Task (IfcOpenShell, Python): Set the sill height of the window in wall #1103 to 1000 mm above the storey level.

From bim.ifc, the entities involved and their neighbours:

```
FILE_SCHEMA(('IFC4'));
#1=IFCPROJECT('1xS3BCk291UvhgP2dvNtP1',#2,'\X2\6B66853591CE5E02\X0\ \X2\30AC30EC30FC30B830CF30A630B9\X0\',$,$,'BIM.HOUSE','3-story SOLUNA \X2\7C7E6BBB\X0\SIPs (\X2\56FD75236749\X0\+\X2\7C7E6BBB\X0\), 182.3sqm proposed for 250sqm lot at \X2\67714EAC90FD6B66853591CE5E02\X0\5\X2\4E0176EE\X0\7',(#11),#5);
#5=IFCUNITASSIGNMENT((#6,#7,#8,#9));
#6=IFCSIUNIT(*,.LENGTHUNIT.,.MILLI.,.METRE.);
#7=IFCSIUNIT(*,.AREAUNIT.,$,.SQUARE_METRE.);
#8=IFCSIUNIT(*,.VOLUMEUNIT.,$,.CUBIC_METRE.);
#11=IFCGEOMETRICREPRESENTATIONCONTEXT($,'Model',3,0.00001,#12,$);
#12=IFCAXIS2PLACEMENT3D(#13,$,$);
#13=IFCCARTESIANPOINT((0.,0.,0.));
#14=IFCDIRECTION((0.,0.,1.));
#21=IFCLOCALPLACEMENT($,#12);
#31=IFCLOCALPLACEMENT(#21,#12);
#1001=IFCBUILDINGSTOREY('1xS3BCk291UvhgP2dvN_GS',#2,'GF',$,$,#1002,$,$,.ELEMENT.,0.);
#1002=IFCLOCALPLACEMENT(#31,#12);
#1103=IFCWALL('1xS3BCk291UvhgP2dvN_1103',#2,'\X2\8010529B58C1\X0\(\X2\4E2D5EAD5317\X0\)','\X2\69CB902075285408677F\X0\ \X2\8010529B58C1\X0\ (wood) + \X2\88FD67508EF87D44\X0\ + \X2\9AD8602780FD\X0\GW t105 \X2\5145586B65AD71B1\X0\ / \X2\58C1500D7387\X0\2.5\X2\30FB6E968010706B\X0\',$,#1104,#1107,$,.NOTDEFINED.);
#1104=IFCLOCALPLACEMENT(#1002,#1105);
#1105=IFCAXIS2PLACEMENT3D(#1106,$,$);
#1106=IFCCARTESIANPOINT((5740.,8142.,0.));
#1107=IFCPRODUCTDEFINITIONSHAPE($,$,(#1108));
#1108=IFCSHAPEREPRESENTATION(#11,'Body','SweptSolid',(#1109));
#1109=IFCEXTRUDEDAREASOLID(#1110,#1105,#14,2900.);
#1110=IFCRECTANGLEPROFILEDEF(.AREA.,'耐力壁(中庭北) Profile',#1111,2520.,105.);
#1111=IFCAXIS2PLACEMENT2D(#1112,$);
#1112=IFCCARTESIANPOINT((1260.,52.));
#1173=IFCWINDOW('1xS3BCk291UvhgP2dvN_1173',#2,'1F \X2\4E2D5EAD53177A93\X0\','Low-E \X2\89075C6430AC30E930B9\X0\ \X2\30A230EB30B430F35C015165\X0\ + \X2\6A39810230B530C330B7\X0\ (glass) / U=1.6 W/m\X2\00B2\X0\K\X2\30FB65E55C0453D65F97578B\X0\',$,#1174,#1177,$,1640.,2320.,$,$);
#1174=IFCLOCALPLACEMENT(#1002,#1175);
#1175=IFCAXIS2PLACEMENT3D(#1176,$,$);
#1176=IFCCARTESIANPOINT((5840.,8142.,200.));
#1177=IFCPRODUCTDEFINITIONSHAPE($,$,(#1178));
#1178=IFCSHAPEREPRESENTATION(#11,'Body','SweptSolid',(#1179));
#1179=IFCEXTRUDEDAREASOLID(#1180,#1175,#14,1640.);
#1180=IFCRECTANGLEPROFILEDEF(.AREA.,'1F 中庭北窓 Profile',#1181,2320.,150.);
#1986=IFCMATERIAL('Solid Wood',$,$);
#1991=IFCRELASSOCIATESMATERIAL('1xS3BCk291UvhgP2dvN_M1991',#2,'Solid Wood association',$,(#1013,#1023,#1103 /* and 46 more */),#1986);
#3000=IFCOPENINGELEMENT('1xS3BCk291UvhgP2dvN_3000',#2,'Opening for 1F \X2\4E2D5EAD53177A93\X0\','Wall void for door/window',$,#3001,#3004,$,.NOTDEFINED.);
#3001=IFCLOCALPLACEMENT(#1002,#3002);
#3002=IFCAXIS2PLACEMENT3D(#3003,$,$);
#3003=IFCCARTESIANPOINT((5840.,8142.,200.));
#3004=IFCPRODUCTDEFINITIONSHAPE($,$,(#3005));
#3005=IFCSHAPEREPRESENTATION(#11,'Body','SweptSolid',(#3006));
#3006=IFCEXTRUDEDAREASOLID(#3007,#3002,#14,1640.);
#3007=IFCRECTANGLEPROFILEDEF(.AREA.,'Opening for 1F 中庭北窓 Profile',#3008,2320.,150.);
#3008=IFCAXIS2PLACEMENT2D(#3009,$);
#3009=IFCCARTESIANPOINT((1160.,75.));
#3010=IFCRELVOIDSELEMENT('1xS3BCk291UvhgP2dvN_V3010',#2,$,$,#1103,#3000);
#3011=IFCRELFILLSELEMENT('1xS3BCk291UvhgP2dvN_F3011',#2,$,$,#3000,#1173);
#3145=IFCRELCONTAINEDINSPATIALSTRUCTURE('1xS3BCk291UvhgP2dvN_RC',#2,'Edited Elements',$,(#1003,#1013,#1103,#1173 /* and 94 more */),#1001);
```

```python
import numpy as np
import ifcopenshell
import ifcopenshell.api.geometry
import ifcopenshell.geom
import ifcopenshell.util.element
import ifcopenshell.util.placement
import ifcopenshell.util.shape
import ifcopenshell.util.unit

model = ifcopenshell.open("bim.ifc")
unit_scale = ifcopenshell.util.unit.calculate_unit_scale(model)

window = model.by_guid("1xS3BCk291UvhgP2dvN_1173")
opening = window.FillsVoids[0].RelatingOpeningElement
storey = ifcopenshell.util.element.get_container(window, ifc_class="IfcBuildingStorey")
level = ifcopenshell.util.placement.get_local_placement(storey.ObjectPlacement)[2, 3]

# The opening's origin need not be at the sill, so measure its lowest point.
shape = ifcopenshell.geom.create_shape(ifcopenshell.geom.settings(), opening)
bottom = ifcopenshell.util.shape.get_shape_bottom_elevation(shape, shape.geometry) / unit_scale
dz = level + 1 / unit_scale - bottom

shift = np.array([0.0, 0.0, dz])
# The window is not placed relative to its opening, so move both.
for product in (opening, window):
    matrix = ifcopenshell.util.placement.get_local_placement(product.ObjectPlacement)
    matrix[:3, 3] += shift
    ifcopenshell.api.geometry.edit_object_placement(model, product=product, matrix=matrix, is_si=False)

print(f"moved by {dz * unit_scale:+.3f} m")

model.write("bim_rev.ifc")
```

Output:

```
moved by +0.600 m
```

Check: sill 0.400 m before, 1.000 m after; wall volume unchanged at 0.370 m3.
